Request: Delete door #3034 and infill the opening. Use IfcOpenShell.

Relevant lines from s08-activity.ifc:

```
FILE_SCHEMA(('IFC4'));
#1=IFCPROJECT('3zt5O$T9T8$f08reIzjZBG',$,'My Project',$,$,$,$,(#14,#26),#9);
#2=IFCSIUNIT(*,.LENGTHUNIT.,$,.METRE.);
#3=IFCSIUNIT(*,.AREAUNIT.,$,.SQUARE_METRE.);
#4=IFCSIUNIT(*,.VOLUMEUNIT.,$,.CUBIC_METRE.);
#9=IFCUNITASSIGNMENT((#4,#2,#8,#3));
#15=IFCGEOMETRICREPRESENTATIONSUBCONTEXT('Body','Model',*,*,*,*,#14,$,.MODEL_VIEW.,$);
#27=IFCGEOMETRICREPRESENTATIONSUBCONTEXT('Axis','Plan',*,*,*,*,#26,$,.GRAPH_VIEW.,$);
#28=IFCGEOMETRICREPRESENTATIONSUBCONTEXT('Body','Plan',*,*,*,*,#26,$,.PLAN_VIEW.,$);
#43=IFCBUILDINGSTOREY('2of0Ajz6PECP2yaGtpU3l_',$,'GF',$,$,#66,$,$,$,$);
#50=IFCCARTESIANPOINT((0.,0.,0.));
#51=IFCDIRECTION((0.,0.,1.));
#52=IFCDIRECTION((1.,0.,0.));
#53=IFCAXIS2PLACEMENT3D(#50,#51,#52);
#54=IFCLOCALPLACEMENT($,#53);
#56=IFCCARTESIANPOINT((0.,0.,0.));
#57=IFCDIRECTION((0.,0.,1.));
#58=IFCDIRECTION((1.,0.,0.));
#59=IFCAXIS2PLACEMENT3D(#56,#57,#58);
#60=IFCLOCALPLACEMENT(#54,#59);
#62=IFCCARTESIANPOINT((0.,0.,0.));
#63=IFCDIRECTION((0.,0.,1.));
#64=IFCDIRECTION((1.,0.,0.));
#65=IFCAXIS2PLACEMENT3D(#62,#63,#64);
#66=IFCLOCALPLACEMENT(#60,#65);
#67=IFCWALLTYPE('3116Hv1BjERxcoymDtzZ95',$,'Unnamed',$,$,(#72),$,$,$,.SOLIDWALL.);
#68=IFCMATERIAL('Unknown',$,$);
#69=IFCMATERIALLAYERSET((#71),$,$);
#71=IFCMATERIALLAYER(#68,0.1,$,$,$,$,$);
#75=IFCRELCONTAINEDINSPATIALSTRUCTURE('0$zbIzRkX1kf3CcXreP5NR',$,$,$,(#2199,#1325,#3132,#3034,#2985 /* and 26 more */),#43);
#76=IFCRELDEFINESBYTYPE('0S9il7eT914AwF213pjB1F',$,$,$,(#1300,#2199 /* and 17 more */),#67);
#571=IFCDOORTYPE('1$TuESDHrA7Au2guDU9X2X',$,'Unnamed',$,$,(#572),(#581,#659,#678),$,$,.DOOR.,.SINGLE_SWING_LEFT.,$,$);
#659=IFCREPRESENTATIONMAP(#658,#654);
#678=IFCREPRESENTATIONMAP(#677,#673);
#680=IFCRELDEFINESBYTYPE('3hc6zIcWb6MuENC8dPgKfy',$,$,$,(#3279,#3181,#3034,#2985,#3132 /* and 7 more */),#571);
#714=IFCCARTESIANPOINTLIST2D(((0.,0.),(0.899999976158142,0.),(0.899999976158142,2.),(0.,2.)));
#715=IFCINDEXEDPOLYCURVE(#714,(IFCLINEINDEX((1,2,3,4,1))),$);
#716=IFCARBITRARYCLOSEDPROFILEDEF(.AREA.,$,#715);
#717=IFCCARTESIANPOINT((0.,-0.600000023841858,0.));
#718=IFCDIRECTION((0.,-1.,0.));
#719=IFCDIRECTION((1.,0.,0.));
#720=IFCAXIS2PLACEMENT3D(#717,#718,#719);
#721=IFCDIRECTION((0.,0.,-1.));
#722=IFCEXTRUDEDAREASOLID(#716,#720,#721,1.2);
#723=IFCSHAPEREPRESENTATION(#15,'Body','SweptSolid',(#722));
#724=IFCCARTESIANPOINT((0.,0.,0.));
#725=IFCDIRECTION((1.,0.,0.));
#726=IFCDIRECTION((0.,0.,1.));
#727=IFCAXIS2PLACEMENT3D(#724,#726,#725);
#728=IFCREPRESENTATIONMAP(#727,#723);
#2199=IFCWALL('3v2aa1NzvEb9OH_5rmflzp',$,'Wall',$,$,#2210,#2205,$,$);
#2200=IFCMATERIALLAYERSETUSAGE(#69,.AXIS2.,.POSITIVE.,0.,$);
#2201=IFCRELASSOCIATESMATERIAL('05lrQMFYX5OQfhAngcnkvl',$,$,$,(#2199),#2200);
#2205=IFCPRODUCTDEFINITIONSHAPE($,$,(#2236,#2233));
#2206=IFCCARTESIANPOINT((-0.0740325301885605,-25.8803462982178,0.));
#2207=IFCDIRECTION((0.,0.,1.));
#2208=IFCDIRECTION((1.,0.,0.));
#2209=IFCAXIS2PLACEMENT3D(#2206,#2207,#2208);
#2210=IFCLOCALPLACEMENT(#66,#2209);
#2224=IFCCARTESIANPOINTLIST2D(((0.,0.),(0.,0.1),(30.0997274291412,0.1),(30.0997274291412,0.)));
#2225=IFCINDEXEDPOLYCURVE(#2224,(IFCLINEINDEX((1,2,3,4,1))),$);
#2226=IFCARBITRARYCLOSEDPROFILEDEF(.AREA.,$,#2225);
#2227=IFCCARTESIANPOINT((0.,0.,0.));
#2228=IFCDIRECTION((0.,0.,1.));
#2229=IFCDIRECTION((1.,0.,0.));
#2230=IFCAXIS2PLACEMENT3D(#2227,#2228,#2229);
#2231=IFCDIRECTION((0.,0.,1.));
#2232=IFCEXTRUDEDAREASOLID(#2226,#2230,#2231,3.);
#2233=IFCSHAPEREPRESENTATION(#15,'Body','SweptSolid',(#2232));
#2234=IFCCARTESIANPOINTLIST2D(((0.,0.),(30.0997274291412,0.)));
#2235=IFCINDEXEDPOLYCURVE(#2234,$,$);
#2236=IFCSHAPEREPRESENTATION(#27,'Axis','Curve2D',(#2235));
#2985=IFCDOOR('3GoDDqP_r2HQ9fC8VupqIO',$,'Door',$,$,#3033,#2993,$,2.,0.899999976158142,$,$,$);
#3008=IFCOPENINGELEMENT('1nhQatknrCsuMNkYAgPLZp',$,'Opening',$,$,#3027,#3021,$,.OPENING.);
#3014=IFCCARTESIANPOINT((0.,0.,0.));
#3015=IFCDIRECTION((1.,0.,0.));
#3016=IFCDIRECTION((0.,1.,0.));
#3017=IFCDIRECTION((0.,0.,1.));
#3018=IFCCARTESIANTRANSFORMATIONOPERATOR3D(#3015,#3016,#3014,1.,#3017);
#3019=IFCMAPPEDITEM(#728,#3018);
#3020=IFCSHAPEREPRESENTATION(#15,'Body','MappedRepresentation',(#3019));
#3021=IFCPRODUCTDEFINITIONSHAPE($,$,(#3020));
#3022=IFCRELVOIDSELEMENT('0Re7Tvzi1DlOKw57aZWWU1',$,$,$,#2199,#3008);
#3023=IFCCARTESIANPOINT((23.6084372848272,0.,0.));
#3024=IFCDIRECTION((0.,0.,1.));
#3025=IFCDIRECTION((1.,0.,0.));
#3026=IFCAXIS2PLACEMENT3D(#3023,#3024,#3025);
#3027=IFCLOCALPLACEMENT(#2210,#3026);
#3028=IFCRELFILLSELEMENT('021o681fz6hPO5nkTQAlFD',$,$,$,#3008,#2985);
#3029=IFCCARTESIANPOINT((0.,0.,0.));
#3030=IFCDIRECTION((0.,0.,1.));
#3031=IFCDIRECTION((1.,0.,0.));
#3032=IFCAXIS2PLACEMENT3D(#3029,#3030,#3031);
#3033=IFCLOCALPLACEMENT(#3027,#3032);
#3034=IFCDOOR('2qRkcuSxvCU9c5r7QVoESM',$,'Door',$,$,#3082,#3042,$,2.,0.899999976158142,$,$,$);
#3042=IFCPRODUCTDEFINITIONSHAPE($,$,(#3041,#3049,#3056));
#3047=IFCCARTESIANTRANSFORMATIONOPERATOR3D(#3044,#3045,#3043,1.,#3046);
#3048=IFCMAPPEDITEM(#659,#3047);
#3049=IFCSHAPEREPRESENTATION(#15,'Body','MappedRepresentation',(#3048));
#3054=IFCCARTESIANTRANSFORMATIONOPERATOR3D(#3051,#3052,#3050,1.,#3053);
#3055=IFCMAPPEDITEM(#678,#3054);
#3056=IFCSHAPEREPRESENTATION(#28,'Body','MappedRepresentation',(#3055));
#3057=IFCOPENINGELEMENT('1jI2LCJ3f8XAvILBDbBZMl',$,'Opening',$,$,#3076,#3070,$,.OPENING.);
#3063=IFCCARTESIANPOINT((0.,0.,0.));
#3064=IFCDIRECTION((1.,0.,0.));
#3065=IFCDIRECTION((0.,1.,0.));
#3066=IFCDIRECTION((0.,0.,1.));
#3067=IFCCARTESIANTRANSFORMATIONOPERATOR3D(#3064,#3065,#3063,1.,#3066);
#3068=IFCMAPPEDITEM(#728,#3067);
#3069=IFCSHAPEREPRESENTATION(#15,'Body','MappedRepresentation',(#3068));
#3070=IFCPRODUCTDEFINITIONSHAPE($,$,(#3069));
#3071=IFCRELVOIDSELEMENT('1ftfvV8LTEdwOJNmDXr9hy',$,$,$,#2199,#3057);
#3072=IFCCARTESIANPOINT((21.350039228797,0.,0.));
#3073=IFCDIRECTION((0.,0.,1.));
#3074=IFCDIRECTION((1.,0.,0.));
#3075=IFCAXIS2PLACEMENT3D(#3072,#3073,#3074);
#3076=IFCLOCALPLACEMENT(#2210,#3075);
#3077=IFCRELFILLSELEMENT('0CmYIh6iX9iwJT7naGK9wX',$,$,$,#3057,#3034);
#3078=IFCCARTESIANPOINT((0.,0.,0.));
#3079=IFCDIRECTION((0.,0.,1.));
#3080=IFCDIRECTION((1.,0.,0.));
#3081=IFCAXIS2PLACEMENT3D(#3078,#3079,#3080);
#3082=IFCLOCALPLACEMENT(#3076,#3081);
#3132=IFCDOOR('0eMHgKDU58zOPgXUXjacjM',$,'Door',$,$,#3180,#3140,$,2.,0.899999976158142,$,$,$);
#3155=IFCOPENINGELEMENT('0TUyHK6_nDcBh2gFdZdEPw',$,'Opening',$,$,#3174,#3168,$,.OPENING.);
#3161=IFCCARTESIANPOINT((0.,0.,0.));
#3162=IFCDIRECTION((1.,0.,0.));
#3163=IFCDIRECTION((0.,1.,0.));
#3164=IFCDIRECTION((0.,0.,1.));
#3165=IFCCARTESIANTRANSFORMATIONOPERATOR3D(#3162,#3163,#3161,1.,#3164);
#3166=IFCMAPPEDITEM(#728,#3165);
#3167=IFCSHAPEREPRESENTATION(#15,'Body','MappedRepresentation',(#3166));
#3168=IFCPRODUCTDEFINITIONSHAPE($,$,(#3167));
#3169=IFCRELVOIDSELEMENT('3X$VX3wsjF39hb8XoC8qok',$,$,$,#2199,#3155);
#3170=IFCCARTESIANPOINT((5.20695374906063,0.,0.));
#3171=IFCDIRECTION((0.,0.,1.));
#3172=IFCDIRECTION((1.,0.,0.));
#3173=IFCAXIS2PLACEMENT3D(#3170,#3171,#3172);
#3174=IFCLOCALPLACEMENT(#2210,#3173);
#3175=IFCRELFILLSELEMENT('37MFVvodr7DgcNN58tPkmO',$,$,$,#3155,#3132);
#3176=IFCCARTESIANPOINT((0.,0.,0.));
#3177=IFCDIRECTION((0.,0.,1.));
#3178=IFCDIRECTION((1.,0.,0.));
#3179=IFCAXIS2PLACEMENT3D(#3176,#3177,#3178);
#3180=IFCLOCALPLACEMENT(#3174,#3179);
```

```python
import ifcopenshell
import ifcopenshell.api.feature
import ifcopenshell.api.root
import ifcopenshell.geom
import ifcopenshell.util.shape

model = ifcopenshell.open("s08-activity.ifc")
settings = ifcopenshell.geom.settings()


def volume(element):
    """Net volume in cubic metres, openings subtracted."""
    shape = ifcopenshell.geom.create_shape(settings, element)
    return ifcopenshell.util.shape.get_volume(shape.geometry)


door = model.by_id(3034)
opening = door.FillsVoids[0].RelatingOpeningElement
wall = opening.VoidsElements[0].RelatingBuildingElement
before = volume(wall)

ifcopenshell.api.root.remove_product(model, product=door)
ifcopenshell.api.feature.remove_feature(model, feature=opening)

after = volume(wall)

print(f"wall volume {before:.3f} -> {after:.3f} m3")

model.write("s08-activity_updated.ifc")
```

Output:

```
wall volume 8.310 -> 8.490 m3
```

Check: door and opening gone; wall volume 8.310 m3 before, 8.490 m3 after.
